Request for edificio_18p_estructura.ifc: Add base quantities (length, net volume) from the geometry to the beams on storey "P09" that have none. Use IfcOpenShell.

First a look at what the model holds.

```python
import ifcopenshell
import ifcopenshell.util.element
import ifcopenshell.util.unit

model = ifcopenshell.open("edificio_18p_estructura.ifc")
print(model.schema)
for unit_type in ("LENGTHUNIT", "AREAUNIT", "VOLUMEUNIT"):
    print(unit_type, ifcopenshell.util.unit.calculate_unit_scale(model, unit_type))
storey = next(s for s in model.by_type("IfcBuildingStorey") if s.Name == "P09")
beams = [e for e in ifcopenshell.util.element.get_decomposition(storey) if e.is_a("IfcBeam")]
for e in sorted(beams, key=lambda e: e.id()):
    print(e.id(), e.is_a(), e.Name, list(ifcopenshell.util.element.get_psets(e, qtos_only=True)), sep=" | ")
```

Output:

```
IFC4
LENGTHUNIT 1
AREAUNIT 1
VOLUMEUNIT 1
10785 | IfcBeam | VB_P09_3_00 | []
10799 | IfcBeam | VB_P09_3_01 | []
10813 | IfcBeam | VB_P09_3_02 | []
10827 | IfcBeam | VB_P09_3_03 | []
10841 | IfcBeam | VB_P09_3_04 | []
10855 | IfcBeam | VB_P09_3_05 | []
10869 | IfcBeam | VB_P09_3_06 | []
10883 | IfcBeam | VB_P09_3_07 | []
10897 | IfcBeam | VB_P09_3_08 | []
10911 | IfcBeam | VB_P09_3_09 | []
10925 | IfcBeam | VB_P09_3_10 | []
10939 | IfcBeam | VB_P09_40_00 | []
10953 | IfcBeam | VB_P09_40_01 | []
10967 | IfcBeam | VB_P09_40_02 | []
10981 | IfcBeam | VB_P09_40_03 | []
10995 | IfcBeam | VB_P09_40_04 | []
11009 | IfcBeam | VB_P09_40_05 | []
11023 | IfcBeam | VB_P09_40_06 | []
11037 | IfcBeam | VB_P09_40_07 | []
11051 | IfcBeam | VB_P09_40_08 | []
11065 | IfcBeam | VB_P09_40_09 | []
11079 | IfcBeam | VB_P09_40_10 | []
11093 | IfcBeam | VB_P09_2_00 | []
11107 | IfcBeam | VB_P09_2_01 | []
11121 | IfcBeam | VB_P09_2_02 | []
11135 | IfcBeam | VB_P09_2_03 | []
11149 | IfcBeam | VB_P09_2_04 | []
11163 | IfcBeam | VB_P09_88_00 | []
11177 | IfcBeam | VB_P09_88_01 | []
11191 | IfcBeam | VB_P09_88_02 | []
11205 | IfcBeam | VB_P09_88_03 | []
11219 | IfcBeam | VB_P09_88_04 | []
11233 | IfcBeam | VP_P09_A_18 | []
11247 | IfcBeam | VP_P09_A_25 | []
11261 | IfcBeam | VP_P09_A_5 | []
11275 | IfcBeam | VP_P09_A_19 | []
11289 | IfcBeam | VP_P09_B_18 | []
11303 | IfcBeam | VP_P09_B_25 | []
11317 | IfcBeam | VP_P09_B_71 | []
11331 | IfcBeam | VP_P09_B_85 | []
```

```python
import ifcopenshell
import ifcopenshell.api.pset
import ifcopenshell.geom
import ifcopenshell.util.element
import ifcopenshell.util.shape
import ifcopenshell.util.unit

model = ifcopenshell.open("edificio_18p_estructura.ifc")
unit_scale = ifcopenshell.util.unit.calculate_unit_scale(model)
volume_scale = ifcopenshell.util.unit.calculate_unit_scale(model, "VOLUMEUNIT")
settings = ifcopenshell.geom.settings()

storey = next(s for s in model.by_type("IfcBuildingStorey") if s.Name == "P09")
beams = [e for e in ifcopenshell.util.element.get_decomposition(storey) if e.is_a("IfcBeam")]

for e in sorted(beams, key=lambda e: e.id()):
    if ifcopenshell.util.element.get_psets(e, qtos_only=True, should_inherit=False):
        continue
    # Geometry comes back in metres, in the element's own axes.
    shape = ifcopenshell.geom.create_shape(settings, e)
    values = {
        "Length": ifcopenshell.util.shape.get_max_xyz(shape.geometry) / unit_scale,
        "NetVolume": ifcopenshell.util.shape.get_volume(shape.geometry) / volume_scale,
    }
    qto = ifcopenshell.api.pset.add_qto(model, product=e, name="Qto_BeamBaseQuantities")
    ifcopenshell.api.pset.edit_qto(model, qto=qto, properties=values)
    print(e.id(), {k: round(v, 3) for k, v in values.items()})

model.write("edificio_18p_estructura_rev.ifc")
```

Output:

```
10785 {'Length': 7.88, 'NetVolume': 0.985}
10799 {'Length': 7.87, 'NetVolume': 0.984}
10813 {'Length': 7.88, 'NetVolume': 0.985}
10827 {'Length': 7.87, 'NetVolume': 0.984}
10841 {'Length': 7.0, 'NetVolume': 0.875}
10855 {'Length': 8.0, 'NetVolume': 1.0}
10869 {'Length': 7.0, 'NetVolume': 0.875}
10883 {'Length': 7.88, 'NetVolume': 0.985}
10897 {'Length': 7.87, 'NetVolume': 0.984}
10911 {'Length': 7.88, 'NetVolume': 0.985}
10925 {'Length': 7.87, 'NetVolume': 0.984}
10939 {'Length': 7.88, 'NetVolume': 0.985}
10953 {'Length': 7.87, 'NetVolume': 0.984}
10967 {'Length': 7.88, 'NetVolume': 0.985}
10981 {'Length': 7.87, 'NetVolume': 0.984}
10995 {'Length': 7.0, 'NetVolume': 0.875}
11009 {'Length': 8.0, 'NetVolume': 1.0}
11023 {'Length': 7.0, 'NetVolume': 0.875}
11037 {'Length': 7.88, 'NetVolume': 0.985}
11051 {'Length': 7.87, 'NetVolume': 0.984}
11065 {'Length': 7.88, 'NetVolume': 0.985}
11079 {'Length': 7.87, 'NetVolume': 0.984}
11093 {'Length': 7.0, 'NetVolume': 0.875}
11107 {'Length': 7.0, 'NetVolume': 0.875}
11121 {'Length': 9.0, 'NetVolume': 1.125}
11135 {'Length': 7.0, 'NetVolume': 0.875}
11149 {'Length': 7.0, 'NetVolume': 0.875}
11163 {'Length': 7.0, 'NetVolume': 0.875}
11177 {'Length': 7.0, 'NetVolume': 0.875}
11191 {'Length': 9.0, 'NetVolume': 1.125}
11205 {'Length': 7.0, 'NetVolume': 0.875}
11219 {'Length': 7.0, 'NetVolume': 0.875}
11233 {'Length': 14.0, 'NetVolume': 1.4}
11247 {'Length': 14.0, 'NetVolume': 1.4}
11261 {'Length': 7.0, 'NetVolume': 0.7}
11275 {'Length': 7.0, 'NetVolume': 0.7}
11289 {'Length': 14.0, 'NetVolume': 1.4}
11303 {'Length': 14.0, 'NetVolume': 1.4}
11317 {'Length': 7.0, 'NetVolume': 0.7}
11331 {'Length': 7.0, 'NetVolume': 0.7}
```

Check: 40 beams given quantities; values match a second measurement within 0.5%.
